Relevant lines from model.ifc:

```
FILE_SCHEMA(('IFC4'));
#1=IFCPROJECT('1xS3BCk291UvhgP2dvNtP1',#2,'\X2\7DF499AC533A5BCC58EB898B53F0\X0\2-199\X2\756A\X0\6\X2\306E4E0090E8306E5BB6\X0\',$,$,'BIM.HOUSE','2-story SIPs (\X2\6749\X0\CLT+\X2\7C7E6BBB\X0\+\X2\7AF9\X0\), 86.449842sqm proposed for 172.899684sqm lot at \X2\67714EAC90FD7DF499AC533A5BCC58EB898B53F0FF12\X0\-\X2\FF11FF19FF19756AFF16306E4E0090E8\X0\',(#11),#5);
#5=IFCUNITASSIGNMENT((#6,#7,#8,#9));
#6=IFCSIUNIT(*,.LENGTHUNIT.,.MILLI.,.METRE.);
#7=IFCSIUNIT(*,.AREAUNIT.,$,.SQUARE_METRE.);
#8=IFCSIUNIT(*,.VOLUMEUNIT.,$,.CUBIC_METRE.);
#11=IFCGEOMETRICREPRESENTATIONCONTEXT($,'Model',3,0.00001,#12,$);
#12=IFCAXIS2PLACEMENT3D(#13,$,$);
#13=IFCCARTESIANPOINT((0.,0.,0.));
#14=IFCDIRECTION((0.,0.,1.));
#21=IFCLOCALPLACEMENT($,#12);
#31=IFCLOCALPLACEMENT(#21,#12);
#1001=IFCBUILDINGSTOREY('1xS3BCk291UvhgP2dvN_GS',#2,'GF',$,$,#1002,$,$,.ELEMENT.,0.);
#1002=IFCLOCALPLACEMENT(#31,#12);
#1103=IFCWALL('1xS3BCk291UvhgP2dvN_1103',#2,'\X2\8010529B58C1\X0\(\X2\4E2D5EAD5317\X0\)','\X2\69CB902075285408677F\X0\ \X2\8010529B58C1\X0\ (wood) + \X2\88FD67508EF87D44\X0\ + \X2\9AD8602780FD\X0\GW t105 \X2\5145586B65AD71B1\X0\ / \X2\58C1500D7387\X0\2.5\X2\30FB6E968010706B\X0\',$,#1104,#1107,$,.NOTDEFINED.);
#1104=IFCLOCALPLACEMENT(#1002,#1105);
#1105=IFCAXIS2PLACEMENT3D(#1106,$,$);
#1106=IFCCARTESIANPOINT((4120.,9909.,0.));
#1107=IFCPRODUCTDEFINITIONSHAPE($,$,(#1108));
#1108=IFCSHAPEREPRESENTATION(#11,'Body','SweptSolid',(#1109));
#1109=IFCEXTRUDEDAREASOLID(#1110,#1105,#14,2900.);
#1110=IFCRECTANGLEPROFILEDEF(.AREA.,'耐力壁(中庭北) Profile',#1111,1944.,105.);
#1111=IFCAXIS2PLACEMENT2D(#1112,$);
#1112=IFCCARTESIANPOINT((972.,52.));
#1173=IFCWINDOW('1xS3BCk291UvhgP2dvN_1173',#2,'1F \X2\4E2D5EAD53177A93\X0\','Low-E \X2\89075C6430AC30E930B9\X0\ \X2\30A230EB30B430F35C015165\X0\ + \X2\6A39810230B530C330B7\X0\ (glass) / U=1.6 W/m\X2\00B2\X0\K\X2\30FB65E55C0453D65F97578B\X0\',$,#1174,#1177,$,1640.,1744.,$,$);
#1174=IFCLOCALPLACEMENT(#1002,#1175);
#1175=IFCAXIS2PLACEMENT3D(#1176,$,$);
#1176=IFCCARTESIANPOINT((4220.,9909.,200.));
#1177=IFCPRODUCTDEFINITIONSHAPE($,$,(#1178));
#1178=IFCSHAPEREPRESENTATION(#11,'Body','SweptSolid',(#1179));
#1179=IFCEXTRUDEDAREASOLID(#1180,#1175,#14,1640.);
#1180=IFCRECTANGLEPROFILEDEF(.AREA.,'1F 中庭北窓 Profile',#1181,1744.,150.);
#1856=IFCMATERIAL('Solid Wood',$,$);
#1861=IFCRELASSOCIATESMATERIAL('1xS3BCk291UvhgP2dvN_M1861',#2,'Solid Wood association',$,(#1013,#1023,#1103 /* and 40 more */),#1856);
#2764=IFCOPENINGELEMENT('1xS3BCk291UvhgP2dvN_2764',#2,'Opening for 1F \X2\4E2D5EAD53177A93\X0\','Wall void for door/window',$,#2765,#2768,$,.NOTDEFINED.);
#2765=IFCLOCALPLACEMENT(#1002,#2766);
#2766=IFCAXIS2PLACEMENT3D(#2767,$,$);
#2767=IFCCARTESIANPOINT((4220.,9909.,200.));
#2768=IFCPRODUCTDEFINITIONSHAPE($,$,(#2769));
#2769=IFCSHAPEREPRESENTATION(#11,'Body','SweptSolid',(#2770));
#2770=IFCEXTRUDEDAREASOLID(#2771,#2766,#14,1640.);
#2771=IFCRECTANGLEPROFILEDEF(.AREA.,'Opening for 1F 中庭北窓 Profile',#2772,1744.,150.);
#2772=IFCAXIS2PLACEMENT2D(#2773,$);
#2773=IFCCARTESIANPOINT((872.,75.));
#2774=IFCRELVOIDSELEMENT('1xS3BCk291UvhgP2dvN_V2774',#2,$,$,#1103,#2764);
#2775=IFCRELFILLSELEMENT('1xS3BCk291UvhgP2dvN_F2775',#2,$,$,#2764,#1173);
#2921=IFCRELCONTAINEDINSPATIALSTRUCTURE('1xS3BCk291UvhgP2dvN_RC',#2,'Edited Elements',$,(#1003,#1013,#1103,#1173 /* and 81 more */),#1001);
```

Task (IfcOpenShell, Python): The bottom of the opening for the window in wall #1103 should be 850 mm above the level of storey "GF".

```python
import numpy as np
import ifcopenshell
import ifcopenshell.api.geometry
import ifcopenshell.geom
import ifcopenshell.util.element
import ifcopenshell.util.placement
import ifcopenshell.util.shape
import ifcopenshell.util.unit

model = ifcopenshell.open("model.ifc")
unit_scale = ifcopenshell.util.unit.calculate_unit_scale(model)

window = model.by_guid("1xS3BCk291UvhgP2dvN_1173")
opening = window.FillsVoids[0].RelatingOpeningElement
storey = ifcopenshell.util.element.get_container(window, ifc_class="IfcBuildingStorey")
level = ifcopenshell.util.placement.get_local_placement(storey.ObjectPlacement)[2, 3]

# The opening's origin need not be at the sill, so measure its lowest point.
shape = ifcopenshell.geom.create_shape(ifcopenshell.geom.settings(), opening)
bottom = ifcopenshell.util.shape.get_shape_bottom_elevation(shape, shape.geometry) / unit_scale
dz = level + 0.85 / unit_scale - bottom

shift = np.array([0.0, 0.0, dz])
# The window is not placed relative to its opening, so move both.
for product in (opening, window):
    matrix = ifcopenshell.util.placement.get_local_placement(product.ObjectPlacement)
    matrix[:3, 3] += shift
    ifcopenshell.api.geometry.edit_object_placement(model, product=product, matrix=matrix, is_si=False)

print(f"moved by {dz * unit_scale:+.3f} m")

model.write("model_rev.ifc")
```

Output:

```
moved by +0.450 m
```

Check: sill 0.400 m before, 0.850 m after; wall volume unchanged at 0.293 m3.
